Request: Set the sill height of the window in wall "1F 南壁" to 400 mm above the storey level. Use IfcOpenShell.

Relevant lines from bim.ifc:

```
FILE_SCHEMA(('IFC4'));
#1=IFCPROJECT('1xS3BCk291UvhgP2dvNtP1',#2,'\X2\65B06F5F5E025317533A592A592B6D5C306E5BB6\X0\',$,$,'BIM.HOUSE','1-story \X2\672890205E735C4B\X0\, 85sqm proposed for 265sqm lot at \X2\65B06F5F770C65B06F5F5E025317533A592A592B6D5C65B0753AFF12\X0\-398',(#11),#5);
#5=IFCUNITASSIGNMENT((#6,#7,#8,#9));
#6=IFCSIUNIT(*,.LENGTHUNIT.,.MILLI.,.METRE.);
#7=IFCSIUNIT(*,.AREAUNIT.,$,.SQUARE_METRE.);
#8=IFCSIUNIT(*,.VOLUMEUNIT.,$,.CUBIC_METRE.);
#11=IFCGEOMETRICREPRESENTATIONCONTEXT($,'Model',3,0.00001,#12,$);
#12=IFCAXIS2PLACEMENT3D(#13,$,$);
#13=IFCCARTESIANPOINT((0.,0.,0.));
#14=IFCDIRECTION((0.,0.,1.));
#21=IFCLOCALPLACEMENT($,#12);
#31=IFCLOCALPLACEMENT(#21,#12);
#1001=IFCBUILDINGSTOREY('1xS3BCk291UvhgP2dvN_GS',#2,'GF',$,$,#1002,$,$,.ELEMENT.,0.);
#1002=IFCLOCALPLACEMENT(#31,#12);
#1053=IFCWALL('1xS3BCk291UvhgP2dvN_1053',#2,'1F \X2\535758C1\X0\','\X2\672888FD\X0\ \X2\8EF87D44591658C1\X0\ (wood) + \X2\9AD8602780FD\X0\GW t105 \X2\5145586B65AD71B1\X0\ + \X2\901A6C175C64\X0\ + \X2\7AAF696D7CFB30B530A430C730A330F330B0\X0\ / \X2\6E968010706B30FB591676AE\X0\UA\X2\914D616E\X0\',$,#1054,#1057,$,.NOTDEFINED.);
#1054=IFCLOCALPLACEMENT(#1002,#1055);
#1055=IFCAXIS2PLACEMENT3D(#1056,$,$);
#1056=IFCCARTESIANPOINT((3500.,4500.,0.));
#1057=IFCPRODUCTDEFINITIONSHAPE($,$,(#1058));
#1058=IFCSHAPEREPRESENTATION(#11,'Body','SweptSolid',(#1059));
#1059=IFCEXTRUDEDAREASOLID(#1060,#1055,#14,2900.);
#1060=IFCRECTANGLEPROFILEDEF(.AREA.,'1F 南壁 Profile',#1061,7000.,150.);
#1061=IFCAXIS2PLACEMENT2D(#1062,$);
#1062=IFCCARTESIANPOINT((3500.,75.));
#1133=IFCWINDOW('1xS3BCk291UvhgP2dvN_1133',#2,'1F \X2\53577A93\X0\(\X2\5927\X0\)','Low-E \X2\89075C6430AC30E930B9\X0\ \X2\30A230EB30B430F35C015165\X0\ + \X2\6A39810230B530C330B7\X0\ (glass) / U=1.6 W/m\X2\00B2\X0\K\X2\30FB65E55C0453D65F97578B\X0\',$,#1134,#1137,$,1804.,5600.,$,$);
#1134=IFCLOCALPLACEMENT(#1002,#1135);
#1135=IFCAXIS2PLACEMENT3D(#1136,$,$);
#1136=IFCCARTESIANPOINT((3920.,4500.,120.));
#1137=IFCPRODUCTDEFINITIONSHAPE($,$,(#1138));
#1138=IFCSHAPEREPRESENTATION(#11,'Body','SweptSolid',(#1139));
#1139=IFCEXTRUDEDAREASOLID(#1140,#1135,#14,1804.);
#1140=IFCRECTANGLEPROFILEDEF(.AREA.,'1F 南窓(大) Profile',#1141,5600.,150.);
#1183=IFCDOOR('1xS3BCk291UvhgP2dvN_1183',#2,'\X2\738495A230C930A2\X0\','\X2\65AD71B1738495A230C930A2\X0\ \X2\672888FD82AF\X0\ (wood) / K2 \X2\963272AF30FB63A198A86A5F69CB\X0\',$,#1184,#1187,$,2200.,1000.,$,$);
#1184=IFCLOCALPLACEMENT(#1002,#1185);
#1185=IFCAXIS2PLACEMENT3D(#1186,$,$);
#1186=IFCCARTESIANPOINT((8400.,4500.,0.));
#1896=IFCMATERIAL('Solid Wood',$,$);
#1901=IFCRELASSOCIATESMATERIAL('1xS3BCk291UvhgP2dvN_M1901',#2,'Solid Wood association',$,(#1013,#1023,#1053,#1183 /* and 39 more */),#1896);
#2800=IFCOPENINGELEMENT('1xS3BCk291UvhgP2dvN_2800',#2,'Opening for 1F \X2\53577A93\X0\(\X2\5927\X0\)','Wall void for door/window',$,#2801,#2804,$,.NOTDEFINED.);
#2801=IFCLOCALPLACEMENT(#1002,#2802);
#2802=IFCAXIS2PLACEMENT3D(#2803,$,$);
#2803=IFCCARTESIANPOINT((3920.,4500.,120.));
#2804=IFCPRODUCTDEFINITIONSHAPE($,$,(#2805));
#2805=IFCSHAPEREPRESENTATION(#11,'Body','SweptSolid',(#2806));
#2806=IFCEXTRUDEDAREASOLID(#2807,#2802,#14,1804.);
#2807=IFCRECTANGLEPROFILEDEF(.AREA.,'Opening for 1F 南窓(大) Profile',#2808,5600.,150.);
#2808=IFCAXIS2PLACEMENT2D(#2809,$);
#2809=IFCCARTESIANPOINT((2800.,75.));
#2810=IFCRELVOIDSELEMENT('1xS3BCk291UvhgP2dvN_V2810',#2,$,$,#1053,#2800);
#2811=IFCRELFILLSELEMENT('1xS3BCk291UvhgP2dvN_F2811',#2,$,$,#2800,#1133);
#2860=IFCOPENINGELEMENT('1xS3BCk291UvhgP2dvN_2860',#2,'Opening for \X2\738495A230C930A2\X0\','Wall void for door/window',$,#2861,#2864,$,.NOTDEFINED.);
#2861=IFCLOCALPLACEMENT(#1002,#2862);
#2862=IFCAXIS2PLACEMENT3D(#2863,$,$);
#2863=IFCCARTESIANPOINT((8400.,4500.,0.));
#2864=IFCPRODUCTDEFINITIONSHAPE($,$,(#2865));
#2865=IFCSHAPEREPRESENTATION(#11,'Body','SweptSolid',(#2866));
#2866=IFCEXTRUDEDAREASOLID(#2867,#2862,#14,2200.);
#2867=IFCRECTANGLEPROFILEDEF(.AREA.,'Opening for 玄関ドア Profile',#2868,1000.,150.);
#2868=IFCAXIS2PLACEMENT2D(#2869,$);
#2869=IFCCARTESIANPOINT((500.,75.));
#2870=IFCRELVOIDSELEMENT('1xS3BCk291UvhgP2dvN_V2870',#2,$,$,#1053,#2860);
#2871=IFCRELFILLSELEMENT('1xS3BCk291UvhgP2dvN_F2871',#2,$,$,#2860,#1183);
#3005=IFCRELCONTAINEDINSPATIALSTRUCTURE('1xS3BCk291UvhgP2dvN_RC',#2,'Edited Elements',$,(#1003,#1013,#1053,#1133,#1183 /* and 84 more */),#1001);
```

```python
import numpy as np
import ifcopenshell
import ifcopenshell.api.geometry
import ifcopenshell.geom
import ifcopenshell.util.element
import ifcopenshell.util.placement
import ifcopenshell.util.shape
import ifcopenshell.util.unit

model = ifcopenshell.open("bim.ifc")
unit_scale = ifcopenshell.util.unit.calculate_unit_scale(model)

window = model.by_guid("1xS3BCk291UvhgP2dvN_1133")
opening = window.FillsVoids[0].RelatingOpeningElement
storey = ifcopenshell.util.element.get_container(window, ifc_class="IfcBuildingStorey")
level = ifcopenshell.util.placement.get_local_placement(storey.ObjectPlacement)[2, 3]

# The opening's origin need not be at the sill, so measure its lowest point.
shape = ifcopenshell.geom.create_shape(ifcopenshell.geom.settings(), opening)
bottom = ifcopenshell.util.shape.get_shape_bottom_elevation(shape, shape.geometry) / unit_scale
dz = level + 400.0 - bottom

shift = np.array([0.0, 0.0, dz])
# The window is not placed relative to its opening, so move both.
for product in (opening, window):
    matrix = ifcopenshell.util.placement.get_local_placement(product.ObjectPlacement)
    matrix[:3, 3] += shift
    ifcopenshell.api.geometry.edit_object_placement(model, product=product, matrix=matrix, is_si=False)

print(f"moved by {dz * unit_scale:+.3f} m")

model.write("bim_rev.ifc")
```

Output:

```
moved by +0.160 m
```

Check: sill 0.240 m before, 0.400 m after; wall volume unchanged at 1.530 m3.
